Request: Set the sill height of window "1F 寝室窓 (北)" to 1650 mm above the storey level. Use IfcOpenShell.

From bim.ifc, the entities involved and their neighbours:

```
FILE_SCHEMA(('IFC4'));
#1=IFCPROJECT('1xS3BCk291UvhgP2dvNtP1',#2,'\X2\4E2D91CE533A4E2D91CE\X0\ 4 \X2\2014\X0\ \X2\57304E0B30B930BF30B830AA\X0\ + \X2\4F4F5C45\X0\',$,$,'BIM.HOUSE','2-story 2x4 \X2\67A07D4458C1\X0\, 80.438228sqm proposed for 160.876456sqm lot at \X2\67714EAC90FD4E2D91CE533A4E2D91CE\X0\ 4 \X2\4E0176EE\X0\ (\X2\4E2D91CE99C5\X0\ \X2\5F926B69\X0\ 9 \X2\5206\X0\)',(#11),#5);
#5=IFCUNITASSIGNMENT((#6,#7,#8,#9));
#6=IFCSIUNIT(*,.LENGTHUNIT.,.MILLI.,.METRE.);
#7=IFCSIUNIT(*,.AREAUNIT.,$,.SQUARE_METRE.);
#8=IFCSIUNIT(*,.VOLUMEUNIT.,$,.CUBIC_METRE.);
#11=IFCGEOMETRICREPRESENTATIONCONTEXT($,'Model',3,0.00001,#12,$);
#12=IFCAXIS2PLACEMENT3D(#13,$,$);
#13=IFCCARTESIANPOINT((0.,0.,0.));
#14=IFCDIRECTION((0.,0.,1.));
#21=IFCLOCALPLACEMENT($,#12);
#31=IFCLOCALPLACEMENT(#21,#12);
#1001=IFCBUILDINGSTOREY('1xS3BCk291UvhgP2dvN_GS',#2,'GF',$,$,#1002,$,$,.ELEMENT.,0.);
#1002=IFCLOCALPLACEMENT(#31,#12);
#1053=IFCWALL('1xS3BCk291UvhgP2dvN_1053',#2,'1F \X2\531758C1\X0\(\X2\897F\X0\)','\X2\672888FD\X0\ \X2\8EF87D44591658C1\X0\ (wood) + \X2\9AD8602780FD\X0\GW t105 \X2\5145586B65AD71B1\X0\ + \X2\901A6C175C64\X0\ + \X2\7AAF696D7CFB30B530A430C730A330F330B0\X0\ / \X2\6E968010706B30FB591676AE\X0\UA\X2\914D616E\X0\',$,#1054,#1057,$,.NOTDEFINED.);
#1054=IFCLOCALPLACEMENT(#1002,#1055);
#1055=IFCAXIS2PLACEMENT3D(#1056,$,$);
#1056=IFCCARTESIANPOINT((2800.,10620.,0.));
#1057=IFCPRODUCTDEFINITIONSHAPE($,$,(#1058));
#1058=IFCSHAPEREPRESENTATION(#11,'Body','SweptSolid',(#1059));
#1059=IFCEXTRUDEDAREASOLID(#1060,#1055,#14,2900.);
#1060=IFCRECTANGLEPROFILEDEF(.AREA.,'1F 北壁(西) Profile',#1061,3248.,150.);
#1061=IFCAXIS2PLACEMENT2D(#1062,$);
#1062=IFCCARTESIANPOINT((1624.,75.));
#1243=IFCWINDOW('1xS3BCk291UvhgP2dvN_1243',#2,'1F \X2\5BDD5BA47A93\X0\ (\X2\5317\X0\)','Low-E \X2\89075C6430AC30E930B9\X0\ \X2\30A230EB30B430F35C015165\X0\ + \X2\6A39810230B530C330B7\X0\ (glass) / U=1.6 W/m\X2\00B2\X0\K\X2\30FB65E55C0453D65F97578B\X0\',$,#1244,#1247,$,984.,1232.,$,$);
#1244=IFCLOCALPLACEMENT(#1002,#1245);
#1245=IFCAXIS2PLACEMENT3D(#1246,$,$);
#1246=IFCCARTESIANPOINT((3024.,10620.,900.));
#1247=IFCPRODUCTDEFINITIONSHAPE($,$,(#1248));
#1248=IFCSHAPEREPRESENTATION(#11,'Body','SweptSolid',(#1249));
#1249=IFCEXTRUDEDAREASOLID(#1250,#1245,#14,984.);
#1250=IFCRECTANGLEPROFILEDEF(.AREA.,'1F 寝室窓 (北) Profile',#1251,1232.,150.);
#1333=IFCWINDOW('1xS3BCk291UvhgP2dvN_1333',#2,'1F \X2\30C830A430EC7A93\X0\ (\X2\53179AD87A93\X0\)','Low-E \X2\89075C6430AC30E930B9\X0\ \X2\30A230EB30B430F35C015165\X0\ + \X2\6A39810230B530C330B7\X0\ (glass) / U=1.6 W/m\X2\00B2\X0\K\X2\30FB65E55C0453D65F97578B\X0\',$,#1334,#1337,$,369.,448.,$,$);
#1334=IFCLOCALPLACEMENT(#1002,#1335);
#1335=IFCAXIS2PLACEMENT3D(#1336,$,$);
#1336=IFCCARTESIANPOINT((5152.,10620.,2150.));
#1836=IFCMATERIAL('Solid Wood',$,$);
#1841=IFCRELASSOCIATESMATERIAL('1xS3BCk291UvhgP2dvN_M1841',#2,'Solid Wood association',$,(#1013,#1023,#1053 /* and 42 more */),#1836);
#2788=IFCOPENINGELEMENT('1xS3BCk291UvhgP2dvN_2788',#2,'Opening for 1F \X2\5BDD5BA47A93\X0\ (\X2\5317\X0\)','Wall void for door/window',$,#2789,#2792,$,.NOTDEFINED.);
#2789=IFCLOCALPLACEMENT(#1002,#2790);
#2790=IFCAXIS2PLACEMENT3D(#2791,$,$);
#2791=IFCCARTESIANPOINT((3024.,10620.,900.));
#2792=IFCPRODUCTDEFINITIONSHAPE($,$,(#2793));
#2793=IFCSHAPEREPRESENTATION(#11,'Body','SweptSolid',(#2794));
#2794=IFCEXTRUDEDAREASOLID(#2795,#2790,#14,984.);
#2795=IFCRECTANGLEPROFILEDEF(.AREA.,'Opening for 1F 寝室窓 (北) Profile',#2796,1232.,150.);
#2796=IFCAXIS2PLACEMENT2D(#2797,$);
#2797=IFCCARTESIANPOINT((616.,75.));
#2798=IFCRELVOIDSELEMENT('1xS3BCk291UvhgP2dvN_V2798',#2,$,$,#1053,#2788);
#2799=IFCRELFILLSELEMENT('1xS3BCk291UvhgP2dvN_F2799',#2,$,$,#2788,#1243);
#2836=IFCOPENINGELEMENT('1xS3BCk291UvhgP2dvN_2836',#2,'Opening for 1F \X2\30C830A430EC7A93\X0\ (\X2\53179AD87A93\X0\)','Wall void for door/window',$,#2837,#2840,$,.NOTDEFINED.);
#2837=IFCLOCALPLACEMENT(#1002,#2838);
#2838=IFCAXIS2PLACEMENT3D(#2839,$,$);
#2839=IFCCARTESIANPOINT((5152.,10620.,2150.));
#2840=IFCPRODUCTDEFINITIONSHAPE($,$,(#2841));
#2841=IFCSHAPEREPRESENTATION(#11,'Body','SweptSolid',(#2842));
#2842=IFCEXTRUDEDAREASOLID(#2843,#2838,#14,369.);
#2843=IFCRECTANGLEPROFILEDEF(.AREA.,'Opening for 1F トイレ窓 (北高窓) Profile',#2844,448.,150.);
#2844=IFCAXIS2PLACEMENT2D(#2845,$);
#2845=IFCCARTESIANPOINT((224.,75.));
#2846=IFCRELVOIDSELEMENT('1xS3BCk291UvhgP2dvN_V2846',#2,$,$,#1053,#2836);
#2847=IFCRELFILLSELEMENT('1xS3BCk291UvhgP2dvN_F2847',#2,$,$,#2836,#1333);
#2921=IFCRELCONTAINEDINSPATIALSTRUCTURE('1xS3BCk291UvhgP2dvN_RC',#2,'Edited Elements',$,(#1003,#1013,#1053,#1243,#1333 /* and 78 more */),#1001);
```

```python
import numpy as np
import ifcopenshell
import ifcopenshell.api.geometry
import ifcopenshell.geom
import ifcopenshell.util.element
import ifcopenshell.util.placement
import ifcopenshell.util.shape
import ifcopenshell.util.unit

model = ifcopenshell.open("bim.ifc")
unit_scale = ifcopenshell.util.unit.calculate_unit_scale(model)

window = model.by_guid("1xS3BCk291UvhgP2dvN_1243")
opening = window.FillsVoids[0].RelatingOpeningElement
storey = ifcopenshell.util.element.get_container(window, ifc_class="IfcBuildingStorey")
level = ifcopenshell.util.placement.get_local_placement(storey.ObjectPlacement)[2, 3]

# The opening's origin need not be at the sill, so measure its lowest point.
shape = ifcopenshell.geom.create_shape(ifcopenshell.geom.settings(), opening)
bottom = ifcopenshell.util.shape.get_shape_bottom_elevation(shape, shape.geometry) / unit_scale
dz = level + 1.65 / unit_scale - bottom

shift = np.array([0.0, 0.0, dz])
# The window is not placed relative to its opening, so move both.
for product in (opening, window):
    matrix = ifcopenshell.util.placement.get_local_placement(product.ObjectPlacement)
    matrix[:3, 3] += shift
    ifcopenshell.api.geometry.edit_object_placement(model, product=product, matrix=matrix, is_si=False)

print(f"moved by {dz * unit_scale:+.3f} m")

model.write("bim_v2.ifc")
```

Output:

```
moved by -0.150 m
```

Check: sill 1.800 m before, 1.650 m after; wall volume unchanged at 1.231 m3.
